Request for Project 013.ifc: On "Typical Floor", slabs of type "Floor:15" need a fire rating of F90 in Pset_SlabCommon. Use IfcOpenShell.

First a look at what the model holds.

```python
import ifcopenshell
import ifcopenshell.util.element

model = ifcopenshell.open("Project 013.ifc")
print(model.schema)
storey = next(s for s in model.by_type("IfcBuildingStorey") if s.Name == "Typical Floor")
slabs = [e for e in ifcopenshell.util.element.get_decomposition(storey) if e.is_a("IfcSlab")]
seen = {}
for e in slabs:
    element_type = ifcopenshell.util.element.get_type(e)
    key = (element_type.Name if element_type != e and element_type else None, ifcopenshell.util.element.get_pset(e, "Pset_SlabCommon", "FireRating"))
    seen[key] = seen.get(key, 0) + 1
for (name, value), count in sorted(seen.items(), key=str):
    print(count, "x", name, "|", value)
```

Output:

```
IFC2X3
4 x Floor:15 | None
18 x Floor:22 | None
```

```python
import ifcopenshell
import ifcopenshell.api.pset
import ifcopenshell.util.element

model = ifcopenshell.open("Project 013.ifc")

storey = next(s for s in model.by_type("IfcBuildingStorey") if s.Name == "Typical Floor")
slabs = [e for e in ifcopenshell.util.element.get_decomposition(storey) if e.is_a("IfcSlab")]

count = 0
for e in slabs:
    element_type = ifcopenshell.util.element.get_type(e)
    if element_type in (None, e) or element_type.Name != "Floor:15":
        continue
    # add_pset returns the element's existing set when there is one.
    pset = ifcopenshell.api.pset.add_pset(model, product=e, name="Pset_SlabCommon")
    ifcopenshell.api.pset.edit_pset(model, pset=pset, properties={"FireRating": "F90"})
    count += 1

print(count, "slabs updated")

model.write("Project 013-out.ifc")
```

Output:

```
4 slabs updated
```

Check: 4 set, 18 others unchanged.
